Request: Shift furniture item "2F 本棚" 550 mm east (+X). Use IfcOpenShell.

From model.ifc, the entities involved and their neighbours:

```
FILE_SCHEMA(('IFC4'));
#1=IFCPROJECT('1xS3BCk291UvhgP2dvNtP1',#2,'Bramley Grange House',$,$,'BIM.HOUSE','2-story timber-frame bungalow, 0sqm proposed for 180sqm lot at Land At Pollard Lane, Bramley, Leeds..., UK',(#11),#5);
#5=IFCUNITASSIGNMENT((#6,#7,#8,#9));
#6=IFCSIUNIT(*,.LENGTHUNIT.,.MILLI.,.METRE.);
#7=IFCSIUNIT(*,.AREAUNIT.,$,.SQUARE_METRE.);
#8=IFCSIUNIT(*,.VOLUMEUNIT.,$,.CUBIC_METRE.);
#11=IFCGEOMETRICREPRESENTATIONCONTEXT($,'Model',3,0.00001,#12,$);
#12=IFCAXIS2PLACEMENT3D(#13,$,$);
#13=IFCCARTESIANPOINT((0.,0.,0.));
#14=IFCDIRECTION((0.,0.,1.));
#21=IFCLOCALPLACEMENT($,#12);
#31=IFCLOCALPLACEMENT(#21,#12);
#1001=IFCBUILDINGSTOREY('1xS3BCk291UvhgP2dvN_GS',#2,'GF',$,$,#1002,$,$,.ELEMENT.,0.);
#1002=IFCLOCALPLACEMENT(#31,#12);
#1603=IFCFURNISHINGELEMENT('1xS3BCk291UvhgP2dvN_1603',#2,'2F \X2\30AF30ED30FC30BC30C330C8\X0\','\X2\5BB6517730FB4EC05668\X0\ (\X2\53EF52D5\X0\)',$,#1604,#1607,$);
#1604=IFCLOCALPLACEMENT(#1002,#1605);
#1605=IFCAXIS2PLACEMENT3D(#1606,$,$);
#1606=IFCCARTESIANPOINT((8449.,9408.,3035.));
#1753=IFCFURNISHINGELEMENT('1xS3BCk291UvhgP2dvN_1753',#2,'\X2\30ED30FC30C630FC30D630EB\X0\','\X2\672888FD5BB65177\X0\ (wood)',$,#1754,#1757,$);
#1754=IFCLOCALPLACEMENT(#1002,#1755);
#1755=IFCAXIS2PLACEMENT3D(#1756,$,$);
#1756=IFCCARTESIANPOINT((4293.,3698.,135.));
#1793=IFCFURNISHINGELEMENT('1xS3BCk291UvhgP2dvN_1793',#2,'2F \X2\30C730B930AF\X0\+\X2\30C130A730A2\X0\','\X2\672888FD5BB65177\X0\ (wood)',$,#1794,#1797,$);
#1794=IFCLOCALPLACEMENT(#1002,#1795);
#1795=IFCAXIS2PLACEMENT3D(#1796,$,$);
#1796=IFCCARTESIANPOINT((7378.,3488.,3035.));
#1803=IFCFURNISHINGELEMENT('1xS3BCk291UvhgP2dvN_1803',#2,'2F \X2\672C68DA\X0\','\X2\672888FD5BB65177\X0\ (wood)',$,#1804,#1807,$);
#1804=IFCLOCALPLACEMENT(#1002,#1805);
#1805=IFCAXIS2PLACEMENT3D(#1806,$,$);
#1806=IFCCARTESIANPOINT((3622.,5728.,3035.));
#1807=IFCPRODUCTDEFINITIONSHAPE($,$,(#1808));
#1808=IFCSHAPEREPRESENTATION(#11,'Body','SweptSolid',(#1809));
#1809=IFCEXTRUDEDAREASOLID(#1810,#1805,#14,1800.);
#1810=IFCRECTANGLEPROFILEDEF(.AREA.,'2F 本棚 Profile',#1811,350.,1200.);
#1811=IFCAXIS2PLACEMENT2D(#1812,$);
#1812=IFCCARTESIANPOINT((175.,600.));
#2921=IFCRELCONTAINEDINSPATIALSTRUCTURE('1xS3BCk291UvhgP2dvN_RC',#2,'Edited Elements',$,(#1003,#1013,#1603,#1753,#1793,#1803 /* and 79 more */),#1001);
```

```python
import ifcopenshell
import ifcopenshell.api.geometry
import ifcopenshell.util.placement
import ifcopenshell.util.unit

model = ifcopenshell.open("model.ifc")
unit_scale = ifcopenshell.util.unit.calculate_unit_scale(model)

item = model.by_id(1803)
matrix = ifcopenshell.util.placement.get_local_placement(item.ObjectPlacement)
matrix[0, 3] += 0.55 / unit_scale
ifcopenshell.api.geometry.edit_object_placement(model, product=item, matrix=matrix, is_si=False)

print(ifcopenshell.util.placement.get_local_placement(item.ObjectPlacement).round(3) + 0.0)

model.write("model_rev.ifc")
```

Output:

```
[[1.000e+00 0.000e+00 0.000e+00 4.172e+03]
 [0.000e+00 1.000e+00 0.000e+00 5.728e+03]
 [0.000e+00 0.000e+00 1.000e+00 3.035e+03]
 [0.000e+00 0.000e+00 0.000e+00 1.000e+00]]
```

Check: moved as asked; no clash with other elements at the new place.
